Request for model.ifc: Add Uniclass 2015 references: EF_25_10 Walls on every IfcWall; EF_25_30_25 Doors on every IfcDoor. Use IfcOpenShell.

First a look at what the model holds.

```python
import ifcopenshell

model = ifcopenshell.open("model.ifc")
print(model.schema)
print("classifications:", [c.Name for c in model.by_type("IfcClassification")])
for ifc_class in ("IfcDoor", "IfcRoof", "IfcStair", "IfcWall", "IfcWindow"):
    print(ifc_class, len(model.by_type(ifc_class)))
```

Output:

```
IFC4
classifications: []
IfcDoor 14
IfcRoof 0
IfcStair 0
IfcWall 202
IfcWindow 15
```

```python
import ifcopenshell
import ifcopenshell.api.classification

model = ifcopenshell.open("model.ifc")

system = ifcopenshell.api.classification.add_classification(model, classification="Uniclass 2015")

codes = {
    "IfcWall": ("EF_25_10", "Walls"),
    "IfcDoor": ("EF_25_30_25", "Doors"),
}
for ifc_class, (code, name) in codes.items():
    products = model.by_type(ifc_class)
    ifcopenshell.api.classification.add_reference(
        model, products=products, classification=system, identification=code, name=name
    )
    print(code, len(products))

model.write("model_edited.ifc")
```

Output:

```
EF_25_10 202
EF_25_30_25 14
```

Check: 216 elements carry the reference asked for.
